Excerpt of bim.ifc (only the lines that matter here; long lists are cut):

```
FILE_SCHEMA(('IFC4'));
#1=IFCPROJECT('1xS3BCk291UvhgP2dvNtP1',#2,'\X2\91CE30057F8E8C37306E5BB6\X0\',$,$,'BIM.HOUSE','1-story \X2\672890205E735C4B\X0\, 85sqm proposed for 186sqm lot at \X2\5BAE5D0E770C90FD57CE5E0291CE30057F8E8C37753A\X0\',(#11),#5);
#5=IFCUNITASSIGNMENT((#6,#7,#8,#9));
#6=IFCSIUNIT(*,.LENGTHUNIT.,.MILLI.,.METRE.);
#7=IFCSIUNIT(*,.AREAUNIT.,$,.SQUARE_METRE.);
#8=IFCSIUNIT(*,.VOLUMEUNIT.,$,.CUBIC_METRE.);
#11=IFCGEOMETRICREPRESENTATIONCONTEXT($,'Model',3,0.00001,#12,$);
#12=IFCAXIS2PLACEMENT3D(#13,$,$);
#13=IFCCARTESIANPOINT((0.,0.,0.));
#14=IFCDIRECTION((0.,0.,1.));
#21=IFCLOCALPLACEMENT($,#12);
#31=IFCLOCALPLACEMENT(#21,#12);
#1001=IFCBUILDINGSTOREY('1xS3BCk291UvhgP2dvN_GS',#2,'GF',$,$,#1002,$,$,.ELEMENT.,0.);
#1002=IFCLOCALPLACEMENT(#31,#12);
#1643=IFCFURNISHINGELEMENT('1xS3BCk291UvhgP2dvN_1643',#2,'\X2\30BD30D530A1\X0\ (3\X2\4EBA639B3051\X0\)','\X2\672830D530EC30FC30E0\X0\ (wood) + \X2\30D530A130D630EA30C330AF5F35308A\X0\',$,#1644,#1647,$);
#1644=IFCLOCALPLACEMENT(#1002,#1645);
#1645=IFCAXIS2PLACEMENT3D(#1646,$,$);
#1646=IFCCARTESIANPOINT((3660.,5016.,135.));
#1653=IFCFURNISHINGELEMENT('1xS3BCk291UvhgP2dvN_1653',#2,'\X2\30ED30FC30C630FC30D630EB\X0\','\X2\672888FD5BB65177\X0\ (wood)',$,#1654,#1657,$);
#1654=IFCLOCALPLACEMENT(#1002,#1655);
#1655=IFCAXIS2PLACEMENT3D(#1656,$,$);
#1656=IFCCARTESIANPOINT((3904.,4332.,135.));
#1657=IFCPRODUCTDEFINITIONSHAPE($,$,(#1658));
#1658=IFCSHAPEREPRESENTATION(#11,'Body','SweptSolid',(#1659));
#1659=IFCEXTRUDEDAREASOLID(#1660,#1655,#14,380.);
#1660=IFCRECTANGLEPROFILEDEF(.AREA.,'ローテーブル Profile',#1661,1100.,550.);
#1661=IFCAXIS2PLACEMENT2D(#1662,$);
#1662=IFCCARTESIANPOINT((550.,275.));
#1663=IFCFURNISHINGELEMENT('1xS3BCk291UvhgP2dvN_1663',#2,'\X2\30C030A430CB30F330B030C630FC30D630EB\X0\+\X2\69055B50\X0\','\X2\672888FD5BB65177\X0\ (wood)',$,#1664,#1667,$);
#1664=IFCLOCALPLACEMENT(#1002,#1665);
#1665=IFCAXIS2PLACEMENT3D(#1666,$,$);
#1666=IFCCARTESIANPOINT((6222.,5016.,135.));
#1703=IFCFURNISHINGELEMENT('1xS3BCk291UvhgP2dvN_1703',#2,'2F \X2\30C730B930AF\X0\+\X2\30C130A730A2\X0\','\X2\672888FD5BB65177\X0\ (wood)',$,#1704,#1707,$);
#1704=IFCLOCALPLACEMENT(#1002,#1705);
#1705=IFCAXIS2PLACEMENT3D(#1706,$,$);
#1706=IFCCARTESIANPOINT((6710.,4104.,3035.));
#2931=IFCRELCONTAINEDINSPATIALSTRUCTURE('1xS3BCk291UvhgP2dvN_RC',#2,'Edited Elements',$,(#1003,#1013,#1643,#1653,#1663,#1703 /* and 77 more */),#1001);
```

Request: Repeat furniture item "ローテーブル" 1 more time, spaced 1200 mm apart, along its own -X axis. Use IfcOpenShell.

```python
import ifcopenshell
import ifcopenshell.api.geometry
import ifcopenshell.api.root
import ifcopenshell.util.element
import ifcopenshell.util.placement

model = ifcopenshell.open("bim.ifc")


def reuse_history(source, copy):
    """copy_class also copies each property set's owner history, people and application; keep the originals."""
    for rel in copy.IsDefinedBy:
        if rel.is_a("IfcRelDefinesByProperties") and (history := rel.RelatingPropertyDefinition.OwnerHistory):
            rel.RelatingPropertyDefinition.OwnerHistory = source.OwnerHistory
            ifcopenshell.util.element.remove_deep2(model, history)


source = model.by_guid("1xS3BCk291UvhgP2dvN_1653")
base = ifcopenshell.util.placement.get_local_placement(source.ObjectPlacement)
step = -base[:3, 0] * 1200.0

for i in range(1, 2):
    copy = ifcopenshell.api.root.copy_class(model, product=source)
    copy.Representation = ifcopenshell.util.element.copy_deep(
        model, source.Representation, exclude=["IfcGeometricRepresentationContext", "IfcRepresentationMap"]
    )
    reuse_history(source, copy)
    matrix = base.copy()
    matrix[:3, 3] += i * step
    print("added at", matrix[:3, 3].round(3) + 0.0)
    ifcopenshell.api.geometry.edit_object_placement(model, product=copy, matrix=matrix, is_si=False)

model.write("bim_v2.ifc")
```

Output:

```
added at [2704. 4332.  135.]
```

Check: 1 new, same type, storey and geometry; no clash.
